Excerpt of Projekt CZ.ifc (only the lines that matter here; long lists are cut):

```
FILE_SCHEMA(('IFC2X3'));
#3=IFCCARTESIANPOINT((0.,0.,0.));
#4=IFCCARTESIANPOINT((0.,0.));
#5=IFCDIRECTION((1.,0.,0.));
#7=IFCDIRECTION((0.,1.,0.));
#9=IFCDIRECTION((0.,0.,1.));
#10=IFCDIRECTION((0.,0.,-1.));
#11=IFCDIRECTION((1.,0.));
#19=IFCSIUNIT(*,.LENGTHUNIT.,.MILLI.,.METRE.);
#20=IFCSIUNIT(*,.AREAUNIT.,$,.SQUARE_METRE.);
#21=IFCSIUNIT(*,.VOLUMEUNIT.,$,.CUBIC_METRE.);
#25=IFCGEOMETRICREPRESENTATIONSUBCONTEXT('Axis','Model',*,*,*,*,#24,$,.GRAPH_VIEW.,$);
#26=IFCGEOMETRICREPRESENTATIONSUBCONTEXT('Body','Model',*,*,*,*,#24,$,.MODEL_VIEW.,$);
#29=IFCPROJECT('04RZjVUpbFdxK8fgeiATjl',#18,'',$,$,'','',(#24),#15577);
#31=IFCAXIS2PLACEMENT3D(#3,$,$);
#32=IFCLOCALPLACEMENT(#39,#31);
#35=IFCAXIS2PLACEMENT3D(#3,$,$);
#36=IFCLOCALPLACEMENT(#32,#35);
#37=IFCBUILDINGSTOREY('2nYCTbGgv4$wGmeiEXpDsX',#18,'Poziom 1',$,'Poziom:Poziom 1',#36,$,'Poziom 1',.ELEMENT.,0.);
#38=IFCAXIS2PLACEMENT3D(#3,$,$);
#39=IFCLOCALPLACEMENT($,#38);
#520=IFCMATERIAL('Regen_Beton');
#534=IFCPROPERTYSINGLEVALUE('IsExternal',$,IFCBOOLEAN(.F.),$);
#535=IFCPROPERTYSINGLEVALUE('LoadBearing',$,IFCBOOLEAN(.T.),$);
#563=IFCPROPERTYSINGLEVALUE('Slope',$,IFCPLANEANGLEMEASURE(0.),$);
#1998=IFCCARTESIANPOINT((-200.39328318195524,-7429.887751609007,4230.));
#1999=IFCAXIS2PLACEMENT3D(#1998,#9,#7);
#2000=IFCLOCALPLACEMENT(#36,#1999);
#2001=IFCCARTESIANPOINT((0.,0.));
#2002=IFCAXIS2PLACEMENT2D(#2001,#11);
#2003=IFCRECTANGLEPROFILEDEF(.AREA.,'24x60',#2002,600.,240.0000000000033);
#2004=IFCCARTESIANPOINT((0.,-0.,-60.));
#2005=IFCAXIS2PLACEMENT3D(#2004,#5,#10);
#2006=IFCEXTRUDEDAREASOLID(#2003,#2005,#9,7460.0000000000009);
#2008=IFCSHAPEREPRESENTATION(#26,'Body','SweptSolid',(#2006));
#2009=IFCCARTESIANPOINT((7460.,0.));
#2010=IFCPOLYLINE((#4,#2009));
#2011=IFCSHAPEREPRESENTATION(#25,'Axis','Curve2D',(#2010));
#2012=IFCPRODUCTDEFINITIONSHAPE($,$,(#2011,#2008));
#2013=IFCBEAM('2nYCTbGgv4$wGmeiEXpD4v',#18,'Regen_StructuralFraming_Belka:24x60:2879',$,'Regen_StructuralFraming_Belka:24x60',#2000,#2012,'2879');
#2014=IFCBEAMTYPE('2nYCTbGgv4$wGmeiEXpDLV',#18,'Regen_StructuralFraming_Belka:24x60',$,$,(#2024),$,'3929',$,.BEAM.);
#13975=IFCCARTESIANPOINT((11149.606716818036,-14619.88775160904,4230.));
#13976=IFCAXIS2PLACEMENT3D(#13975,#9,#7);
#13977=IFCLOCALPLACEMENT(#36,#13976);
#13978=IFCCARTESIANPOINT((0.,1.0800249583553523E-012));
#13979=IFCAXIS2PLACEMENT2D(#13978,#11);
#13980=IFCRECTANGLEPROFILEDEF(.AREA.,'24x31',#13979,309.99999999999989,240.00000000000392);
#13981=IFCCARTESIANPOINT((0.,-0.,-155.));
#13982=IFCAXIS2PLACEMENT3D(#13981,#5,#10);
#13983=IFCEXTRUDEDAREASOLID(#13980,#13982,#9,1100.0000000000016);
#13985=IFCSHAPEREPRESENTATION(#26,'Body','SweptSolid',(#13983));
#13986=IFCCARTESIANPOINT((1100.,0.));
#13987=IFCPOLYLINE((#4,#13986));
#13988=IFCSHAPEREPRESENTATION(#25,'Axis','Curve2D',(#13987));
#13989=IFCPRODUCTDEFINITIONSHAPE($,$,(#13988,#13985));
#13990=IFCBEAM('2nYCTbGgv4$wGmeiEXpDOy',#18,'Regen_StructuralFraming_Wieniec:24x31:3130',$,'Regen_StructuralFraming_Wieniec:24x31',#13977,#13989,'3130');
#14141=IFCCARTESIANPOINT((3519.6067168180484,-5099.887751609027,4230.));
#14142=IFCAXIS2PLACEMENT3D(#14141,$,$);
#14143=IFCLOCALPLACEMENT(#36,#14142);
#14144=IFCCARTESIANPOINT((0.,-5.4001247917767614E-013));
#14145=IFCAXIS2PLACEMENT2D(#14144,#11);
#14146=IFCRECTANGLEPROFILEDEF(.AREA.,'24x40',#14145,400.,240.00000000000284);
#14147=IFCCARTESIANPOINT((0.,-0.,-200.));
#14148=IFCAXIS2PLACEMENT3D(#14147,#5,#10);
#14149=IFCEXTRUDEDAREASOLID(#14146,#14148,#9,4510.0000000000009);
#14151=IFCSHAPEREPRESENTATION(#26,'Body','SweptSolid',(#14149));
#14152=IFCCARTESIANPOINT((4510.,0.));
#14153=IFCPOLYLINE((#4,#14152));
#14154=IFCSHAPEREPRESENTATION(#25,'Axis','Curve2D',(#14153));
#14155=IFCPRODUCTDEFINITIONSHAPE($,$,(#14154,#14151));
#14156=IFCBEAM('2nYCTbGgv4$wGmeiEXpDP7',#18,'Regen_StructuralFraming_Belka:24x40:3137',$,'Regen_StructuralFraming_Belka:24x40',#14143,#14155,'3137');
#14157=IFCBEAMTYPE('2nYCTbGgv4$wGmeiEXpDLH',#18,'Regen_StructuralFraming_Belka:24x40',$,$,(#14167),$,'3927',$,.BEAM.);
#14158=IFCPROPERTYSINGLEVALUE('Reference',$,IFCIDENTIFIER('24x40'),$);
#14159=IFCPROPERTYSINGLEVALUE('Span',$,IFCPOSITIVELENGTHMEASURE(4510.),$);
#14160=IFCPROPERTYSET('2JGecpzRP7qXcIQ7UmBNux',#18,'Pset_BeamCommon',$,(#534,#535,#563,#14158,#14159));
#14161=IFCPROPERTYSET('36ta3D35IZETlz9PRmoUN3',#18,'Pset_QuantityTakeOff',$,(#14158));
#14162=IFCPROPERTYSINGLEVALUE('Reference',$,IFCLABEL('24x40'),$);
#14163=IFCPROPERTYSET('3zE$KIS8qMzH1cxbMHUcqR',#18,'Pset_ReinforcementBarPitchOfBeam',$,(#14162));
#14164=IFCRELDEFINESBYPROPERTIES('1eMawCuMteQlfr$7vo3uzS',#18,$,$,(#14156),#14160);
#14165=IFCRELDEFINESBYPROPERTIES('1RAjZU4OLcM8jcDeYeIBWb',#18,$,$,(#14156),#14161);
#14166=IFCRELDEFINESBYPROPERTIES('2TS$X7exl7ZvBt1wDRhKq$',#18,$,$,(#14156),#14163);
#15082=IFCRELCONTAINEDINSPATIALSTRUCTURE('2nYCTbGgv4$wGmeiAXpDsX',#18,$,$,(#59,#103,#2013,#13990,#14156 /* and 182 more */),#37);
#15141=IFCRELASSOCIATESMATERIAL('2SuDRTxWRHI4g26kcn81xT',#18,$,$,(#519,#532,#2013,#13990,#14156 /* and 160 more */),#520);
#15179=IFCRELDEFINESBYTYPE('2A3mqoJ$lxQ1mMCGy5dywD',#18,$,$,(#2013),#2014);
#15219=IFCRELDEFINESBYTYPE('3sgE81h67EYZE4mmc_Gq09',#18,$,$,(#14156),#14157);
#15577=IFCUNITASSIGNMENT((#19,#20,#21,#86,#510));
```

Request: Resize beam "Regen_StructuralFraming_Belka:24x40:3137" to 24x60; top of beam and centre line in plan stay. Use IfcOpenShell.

```python
import ifcopenshell
import ifcopenshell.api.pset
import ifcopenshell.api.type
import ifcopenshell.util.element
import ifcopenshell.util.representation

model = ifcopenshell.open("Projekt CZ.ifc")

member = model.by_guid("2nYCTbGgv4$wGmeiEXpDP7")
source = next(p for p in model.by_type("IfcRectangleProfileDef") if p.ProfileName == "24x60")

body = ifcopenshell.util.representation.get_representation(member, "Model", "Body")
solid = body.Items[0]
old_profile = solid.SweptArea

# Copy the section's sizes but keep this member's own profile position.
profile = ifcopenshell.util.element.copy(model, source)
# Profiles are centred, so shift by half the change in depth to hold the top.
shift = (old_profile.XDim - profile.XDim) / 2
x, y = old_profile.Position.Location.Coordinates
up = (-1.0, 0.0)  # upwards, in the solid's own plane
location = model.createIfcCartesianPoint((x + up[0] * shift, y + up[1] * shift))
profile.Position = model.createIfcAxis2Placement2D(location, old_profile.Position.RefDirection)
solid.SweptArea = profile
if not model.get_total_inverses(old_profile):
    ifcopenshell.util.element.remove_deep2(model, old_profile)

new_type = model.by_id(2014)
ifcopenshell.api.type.assign_type(
    model, related_objects=[member], relating_type=new_type, should_map_representations=False
)
member.Name = member.Name.replace("24x40", "24x60")
member.ObjectType = "Regen_StructuralFraming_Belka:24x60"
pset = model.by_id(ifcopenshell.util.element.get_pset(member, "Pset_BeamCommon", should_inherit=False)["id"])
ifcopenshell.api.pset.edit_pset(model, pset=pset, properties={"Reference": "24x60"})
pset = model.by_id(ifcopenshell.util.element.get_pset(member, "Pset_QuantityTakeOff", should_inherit=False)["id"])
ifcopenshell.api.pset.edit_pset(model, pset=pset, properties={"Reference": "24x60"})
pset = model.by_id(ifcopenshell.util.element.get_pset(member, "Pset_ReinforcementBarPitchOfBeam", should_inherit=False)["id"])
ifcopenshell.api.pset.edit_pset(model, pset=pset, properties={"Reference": "24x60"})

print(solid.SweptArea)

model.write("Projekt CZ_v2.ifc")
```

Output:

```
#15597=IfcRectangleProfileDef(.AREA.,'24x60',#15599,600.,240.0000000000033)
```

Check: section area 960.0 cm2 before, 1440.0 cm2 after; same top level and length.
